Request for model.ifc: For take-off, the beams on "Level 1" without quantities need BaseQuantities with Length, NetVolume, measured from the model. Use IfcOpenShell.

First a look at what the model holds.

```python
import ifcopenshell
import ifcopenshell.util.element
import ifcopenshell.util.unit

model = ifcopenshell.open("model.ifc")
print(model.schema)
for unit_type in ("LENGTHUNIT", "AREAUNIT", "VOLUMEUNIT"):
    print(unit_type, ifcopenshell.util.unit.calculate_unit_scale(model, unit_type))
storey = next(s for s in model.by_type("IfcBuildingStorey") if s.Name == "Level 1")
beams = [e for e in ifcopenshell.util.element.get_decomposition(storey) if e.is_a("IfcBeam")]
for e in sorted(beams, key=lambda e: e.id()):
    print(e.id(), e.is_a(), e.Name, list(ifcopenshell.util.element.get_psets(e, qtos_only=True)), sep=" | ")
```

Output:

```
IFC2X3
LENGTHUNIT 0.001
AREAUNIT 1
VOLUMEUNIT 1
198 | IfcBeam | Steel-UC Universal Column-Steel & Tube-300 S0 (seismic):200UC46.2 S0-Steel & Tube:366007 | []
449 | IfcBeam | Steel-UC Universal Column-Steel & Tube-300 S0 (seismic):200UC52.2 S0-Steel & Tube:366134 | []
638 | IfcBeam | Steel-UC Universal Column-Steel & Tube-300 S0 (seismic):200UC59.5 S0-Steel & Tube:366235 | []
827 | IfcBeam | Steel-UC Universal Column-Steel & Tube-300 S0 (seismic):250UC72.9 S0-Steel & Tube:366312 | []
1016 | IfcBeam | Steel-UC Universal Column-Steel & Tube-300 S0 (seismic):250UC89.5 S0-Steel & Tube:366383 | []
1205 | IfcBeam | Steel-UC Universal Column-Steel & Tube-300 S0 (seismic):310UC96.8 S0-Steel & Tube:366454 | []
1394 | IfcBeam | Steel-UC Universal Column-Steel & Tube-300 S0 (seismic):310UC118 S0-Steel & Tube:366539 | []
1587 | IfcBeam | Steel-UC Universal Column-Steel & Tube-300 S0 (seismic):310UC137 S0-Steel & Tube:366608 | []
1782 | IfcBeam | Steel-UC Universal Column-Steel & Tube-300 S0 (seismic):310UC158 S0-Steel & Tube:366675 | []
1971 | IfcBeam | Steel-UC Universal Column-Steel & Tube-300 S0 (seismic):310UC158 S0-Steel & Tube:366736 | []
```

```python
import ifcopenshell
import ifcopenshell.api.pset
import ifcopenshell.geom
import ifcopenshell.util.element
import ifcopenshell.util.shape
import ifcopenshell.util.unit

model = ifcopenshell.open("model.ifc")
unit_scale = ifcopenshell.util.unit.calculate_unit_scale(model)
volume_scale = ifcopenshell.util.unit.calculate_unit_scale(model, "VOLUMEUNIT")
settings = ifcopenshell.geom.settings()

storey = next(s for s in model.by_type("IfcBuildingStorey") if s.Name == "Level 1")
beams = [e for e in ifcopenshell.util.element.get_decomposition(storey) if e.is_a("IfcBeam")]

for e in sorted(beams, key=lambda e: e.id()):
    if ifcopenshell.util.element.get_psets(e, qtos_only=True, should_inherit=False):
        continue
    # Geometry comes back in metres, in the element's own axes.
    shape = ifcopenshell.geom.create_shape(settings, e)
    values = {
        "Length": ifcopenshell.util.shape.get_max_xyz(shape.geometry) / unit_scale,
        "NetVolume": ifcopenshell.util.shape.get_volume(shape.geometry) / volume_scale,
    }
    qto = ifcopenshell.api.pset.add_qto(model, product=e, name="BaseQuantities")
    ifcopenshell.api.pset.edit_qto(model, qto=qto, properties=values)
    print(e.id(), {k: round(v, 3) for k, v in values.items()})

model.write("model_rev.ifc")
```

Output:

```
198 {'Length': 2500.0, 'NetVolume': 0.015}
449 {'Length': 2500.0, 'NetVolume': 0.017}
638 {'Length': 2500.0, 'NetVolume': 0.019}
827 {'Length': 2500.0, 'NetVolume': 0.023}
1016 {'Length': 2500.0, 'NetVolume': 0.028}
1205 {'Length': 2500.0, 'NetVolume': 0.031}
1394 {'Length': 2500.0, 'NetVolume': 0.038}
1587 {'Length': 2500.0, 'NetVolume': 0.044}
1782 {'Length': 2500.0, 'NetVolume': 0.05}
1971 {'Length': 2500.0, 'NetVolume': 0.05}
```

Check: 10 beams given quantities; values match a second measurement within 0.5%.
